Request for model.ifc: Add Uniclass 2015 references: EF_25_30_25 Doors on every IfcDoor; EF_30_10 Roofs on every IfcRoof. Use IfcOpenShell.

First a look at what the model holds.

```python
import ifcopenshell

model = ifcopenshell.open("model.ifc")
print(model.schema)
print("classifications:", [c.Name for c in model.by_type("IfcClassification")])
for ifc_class in ("IfcDoor", "IfcRoof", "IfcStair", "IfcWall", "IfcWindow"):
    print(ifc_class, len(model.by_type(ifc_class)))
```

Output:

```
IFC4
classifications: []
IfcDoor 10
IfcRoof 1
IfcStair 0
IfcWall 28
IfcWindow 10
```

```python
import ifcopenshell
import ifcopenshell.api.classification

model = ifcopenshell.open("model.ifc")

system = ifcopenshell.api.classification.add_classification(model, classification="Uniclass 2015")

codes = {
    "IfcDoor": ("EF_25_30_25", "Doors"),
    "IfcRoof": ("EF_30_10", "Roofs"),
}
for ifc_class, (code, name) in codes.items():
    products = model.by_type(ifc_class)
    ifcopenshell.api.classification.add_reference(
        model, products=products, classification=system, identification=code, name=name
    )
    print(code, len(products))

model.write("model_updated.ifc")
```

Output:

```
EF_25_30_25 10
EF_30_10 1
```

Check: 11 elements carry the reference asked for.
